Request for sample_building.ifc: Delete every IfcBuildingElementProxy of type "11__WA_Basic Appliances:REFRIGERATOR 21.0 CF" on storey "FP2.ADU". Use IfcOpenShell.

First a look at what the model holds.

```python
import ifcopenshell
import ifcopenshell.util.element

model = ifcopenshell.open("sample_building.ifc")
print(model.schema)
storey = next(s for s in model.by_type("IfcBuildingStorey") if s.Name == "FP2.ADU")
proxies = [e for e in ifcopenshell.util.element.get_decomposition(storey) if e.is_a("IfcBuildingElementProxy")]
seen = {}
for e in proxies:
    element_type = ifcopenshell.util.element.get_type(e)
    name = element_type.Name if element_type not in (None, e) else None
    seen[name] = seen.get(name, 0) + 1
for name, count in sorted(seen.items(), key=str):
    print(count, "x", name)
```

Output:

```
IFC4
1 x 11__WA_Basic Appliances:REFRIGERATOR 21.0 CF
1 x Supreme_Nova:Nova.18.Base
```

```python
import ifcopenshell
import ifcopenshell.api.root
import ifcopenshell.util.element

model = ifcopenshell.open("sample_building.ifc")

storey = next(s for s in model.by_type("IfcBuildingStorey") if s.Name == "FP2.ADU")
proxies = [e for e in ifcopenshell.util.element.get_decomposition(storey) if e.is_a("IfcBuildingElementProxy")]
targets = [e for e in proxies if (t := ifcopenshell.util.element.get_type(e)) not in (None, e) and t.Name == "11__WA_Basic Appliances:REFRIGERATOR 21.0 CF"]

for e in targets:
    ifcopenshell.api.root.remove_product(model, product=e)
print(len(targets), "removed")

model.write("sample_building-out.ifc")
```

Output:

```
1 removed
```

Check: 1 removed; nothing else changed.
